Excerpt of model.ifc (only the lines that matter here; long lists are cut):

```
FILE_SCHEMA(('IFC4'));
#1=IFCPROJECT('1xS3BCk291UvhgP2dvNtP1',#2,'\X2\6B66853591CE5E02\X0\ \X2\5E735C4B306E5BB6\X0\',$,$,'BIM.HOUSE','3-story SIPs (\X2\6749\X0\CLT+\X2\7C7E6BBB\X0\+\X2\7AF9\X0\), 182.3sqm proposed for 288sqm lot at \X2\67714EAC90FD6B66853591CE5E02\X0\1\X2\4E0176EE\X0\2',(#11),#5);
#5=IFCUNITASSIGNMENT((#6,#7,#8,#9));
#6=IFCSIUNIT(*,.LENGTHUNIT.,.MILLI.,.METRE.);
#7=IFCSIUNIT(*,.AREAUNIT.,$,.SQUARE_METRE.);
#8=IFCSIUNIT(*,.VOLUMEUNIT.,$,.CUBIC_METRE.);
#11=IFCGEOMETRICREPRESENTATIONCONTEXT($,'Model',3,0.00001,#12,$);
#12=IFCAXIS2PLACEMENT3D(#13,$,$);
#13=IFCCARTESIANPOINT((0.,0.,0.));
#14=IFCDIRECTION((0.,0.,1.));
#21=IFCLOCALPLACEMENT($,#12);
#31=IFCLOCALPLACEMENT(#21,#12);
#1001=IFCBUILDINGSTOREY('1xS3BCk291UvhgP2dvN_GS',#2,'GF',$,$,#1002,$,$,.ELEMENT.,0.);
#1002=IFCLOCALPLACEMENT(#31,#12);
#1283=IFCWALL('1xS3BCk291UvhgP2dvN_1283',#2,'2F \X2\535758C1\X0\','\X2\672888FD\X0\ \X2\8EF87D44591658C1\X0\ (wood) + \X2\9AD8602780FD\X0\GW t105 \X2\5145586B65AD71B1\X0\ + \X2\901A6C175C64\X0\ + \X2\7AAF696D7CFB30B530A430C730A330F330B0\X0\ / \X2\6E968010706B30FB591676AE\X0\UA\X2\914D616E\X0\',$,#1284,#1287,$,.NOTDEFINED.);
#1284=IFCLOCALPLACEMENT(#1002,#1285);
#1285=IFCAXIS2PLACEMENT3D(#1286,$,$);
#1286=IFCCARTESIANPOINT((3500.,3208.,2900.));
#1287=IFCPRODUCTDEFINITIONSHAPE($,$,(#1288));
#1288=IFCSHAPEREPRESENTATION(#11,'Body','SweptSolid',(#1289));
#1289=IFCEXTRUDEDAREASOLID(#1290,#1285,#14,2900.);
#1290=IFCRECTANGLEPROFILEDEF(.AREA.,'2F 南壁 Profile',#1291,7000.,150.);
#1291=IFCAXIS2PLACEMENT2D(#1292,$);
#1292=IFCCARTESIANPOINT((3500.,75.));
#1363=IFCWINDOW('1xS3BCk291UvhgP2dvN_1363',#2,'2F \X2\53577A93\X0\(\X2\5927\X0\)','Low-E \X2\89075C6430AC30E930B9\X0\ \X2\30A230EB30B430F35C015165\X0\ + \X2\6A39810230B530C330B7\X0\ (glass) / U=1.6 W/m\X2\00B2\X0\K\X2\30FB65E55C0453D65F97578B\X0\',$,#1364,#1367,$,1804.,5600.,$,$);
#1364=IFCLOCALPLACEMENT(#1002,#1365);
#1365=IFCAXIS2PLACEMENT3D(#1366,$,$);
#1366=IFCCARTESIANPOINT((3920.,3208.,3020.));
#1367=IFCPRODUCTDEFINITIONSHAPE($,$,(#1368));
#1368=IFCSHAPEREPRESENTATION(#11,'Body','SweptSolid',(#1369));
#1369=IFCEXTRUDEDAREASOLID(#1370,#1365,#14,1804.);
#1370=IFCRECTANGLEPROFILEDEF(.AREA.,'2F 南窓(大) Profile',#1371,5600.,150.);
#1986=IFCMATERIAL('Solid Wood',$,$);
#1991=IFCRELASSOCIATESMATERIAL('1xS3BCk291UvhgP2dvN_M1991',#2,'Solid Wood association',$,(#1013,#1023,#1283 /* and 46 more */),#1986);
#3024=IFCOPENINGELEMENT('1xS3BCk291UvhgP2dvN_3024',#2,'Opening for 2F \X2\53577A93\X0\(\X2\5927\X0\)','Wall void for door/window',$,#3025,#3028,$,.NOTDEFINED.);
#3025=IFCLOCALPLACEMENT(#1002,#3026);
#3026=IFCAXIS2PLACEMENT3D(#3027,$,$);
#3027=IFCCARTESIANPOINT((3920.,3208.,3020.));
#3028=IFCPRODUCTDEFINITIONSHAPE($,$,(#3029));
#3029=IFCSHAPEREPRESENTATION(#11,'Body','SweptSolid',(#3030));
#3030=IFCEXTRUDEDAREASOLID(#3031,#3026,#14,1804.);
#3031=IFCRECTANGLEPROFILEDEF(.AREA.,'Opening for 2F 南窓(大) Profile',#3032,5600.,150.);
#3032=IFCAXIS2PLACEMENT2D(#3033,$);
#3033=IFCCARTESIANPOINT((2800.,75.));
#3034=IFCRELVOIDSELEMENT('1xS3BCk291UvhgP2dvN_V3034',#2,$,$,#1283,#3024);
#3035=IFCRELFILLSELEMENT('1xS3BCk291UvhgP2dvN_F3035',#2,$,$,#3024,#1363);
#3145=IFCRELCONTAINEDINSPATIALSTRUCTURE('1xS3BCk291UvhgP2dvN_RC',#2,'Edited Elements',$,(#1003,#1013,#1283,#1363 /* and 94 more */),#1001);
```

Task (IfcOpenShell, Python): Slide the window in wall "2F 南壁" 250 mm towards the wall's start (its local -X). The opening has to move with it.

```python
import ifcopenshell
import ifcopenshell.api.geometry
import ifcopenshell.util.placement
import ifcopenshell.util.unit

model = ifcopenshell.open("model.ifc")
unit_scale = ifcopenshell.util.unit.calculate_unit_scale(model)

window = model.by_guid("1xS3BCk291UvhgP2dvN_1363")
opening = window.FillsVoids[0].RelatingOpeningElement
wall = opening.VoidsElements[0].RelatingBuildingElement

wall_matrix = ifcopenshell.util.placement.get_local_placement(wall.ObjectPlacement)
shift = wall_matrix[:3, 0] * -0.25 / unit_scale
before = ifcopenshell.util.placement.get_local_placement(window.ObjectPlacement)[:3, 3].copy()

# The window is not placed relative to its opening, so move both.
for product in (opening, window):
    matrix = ifcopenshell.util.placement.get_local_placement(product.ObjectPlacement)
    matrix[:3, 3] += shift
    ifcopenshell.api.geometry.edit_object_placement(model, product=product, matrix=matrix, is_si=False)

after = ifcopenshell.util.placement.get_local_placement(window.ObjectPlacement)[:3, 3]
print("window moved by", (after - before).round(3) + 0.0)

model.write("model_v2.ifc")
```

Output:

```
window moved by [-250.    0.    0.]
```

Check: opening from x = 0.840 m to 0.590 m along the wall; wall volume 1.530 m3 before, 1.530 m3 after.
